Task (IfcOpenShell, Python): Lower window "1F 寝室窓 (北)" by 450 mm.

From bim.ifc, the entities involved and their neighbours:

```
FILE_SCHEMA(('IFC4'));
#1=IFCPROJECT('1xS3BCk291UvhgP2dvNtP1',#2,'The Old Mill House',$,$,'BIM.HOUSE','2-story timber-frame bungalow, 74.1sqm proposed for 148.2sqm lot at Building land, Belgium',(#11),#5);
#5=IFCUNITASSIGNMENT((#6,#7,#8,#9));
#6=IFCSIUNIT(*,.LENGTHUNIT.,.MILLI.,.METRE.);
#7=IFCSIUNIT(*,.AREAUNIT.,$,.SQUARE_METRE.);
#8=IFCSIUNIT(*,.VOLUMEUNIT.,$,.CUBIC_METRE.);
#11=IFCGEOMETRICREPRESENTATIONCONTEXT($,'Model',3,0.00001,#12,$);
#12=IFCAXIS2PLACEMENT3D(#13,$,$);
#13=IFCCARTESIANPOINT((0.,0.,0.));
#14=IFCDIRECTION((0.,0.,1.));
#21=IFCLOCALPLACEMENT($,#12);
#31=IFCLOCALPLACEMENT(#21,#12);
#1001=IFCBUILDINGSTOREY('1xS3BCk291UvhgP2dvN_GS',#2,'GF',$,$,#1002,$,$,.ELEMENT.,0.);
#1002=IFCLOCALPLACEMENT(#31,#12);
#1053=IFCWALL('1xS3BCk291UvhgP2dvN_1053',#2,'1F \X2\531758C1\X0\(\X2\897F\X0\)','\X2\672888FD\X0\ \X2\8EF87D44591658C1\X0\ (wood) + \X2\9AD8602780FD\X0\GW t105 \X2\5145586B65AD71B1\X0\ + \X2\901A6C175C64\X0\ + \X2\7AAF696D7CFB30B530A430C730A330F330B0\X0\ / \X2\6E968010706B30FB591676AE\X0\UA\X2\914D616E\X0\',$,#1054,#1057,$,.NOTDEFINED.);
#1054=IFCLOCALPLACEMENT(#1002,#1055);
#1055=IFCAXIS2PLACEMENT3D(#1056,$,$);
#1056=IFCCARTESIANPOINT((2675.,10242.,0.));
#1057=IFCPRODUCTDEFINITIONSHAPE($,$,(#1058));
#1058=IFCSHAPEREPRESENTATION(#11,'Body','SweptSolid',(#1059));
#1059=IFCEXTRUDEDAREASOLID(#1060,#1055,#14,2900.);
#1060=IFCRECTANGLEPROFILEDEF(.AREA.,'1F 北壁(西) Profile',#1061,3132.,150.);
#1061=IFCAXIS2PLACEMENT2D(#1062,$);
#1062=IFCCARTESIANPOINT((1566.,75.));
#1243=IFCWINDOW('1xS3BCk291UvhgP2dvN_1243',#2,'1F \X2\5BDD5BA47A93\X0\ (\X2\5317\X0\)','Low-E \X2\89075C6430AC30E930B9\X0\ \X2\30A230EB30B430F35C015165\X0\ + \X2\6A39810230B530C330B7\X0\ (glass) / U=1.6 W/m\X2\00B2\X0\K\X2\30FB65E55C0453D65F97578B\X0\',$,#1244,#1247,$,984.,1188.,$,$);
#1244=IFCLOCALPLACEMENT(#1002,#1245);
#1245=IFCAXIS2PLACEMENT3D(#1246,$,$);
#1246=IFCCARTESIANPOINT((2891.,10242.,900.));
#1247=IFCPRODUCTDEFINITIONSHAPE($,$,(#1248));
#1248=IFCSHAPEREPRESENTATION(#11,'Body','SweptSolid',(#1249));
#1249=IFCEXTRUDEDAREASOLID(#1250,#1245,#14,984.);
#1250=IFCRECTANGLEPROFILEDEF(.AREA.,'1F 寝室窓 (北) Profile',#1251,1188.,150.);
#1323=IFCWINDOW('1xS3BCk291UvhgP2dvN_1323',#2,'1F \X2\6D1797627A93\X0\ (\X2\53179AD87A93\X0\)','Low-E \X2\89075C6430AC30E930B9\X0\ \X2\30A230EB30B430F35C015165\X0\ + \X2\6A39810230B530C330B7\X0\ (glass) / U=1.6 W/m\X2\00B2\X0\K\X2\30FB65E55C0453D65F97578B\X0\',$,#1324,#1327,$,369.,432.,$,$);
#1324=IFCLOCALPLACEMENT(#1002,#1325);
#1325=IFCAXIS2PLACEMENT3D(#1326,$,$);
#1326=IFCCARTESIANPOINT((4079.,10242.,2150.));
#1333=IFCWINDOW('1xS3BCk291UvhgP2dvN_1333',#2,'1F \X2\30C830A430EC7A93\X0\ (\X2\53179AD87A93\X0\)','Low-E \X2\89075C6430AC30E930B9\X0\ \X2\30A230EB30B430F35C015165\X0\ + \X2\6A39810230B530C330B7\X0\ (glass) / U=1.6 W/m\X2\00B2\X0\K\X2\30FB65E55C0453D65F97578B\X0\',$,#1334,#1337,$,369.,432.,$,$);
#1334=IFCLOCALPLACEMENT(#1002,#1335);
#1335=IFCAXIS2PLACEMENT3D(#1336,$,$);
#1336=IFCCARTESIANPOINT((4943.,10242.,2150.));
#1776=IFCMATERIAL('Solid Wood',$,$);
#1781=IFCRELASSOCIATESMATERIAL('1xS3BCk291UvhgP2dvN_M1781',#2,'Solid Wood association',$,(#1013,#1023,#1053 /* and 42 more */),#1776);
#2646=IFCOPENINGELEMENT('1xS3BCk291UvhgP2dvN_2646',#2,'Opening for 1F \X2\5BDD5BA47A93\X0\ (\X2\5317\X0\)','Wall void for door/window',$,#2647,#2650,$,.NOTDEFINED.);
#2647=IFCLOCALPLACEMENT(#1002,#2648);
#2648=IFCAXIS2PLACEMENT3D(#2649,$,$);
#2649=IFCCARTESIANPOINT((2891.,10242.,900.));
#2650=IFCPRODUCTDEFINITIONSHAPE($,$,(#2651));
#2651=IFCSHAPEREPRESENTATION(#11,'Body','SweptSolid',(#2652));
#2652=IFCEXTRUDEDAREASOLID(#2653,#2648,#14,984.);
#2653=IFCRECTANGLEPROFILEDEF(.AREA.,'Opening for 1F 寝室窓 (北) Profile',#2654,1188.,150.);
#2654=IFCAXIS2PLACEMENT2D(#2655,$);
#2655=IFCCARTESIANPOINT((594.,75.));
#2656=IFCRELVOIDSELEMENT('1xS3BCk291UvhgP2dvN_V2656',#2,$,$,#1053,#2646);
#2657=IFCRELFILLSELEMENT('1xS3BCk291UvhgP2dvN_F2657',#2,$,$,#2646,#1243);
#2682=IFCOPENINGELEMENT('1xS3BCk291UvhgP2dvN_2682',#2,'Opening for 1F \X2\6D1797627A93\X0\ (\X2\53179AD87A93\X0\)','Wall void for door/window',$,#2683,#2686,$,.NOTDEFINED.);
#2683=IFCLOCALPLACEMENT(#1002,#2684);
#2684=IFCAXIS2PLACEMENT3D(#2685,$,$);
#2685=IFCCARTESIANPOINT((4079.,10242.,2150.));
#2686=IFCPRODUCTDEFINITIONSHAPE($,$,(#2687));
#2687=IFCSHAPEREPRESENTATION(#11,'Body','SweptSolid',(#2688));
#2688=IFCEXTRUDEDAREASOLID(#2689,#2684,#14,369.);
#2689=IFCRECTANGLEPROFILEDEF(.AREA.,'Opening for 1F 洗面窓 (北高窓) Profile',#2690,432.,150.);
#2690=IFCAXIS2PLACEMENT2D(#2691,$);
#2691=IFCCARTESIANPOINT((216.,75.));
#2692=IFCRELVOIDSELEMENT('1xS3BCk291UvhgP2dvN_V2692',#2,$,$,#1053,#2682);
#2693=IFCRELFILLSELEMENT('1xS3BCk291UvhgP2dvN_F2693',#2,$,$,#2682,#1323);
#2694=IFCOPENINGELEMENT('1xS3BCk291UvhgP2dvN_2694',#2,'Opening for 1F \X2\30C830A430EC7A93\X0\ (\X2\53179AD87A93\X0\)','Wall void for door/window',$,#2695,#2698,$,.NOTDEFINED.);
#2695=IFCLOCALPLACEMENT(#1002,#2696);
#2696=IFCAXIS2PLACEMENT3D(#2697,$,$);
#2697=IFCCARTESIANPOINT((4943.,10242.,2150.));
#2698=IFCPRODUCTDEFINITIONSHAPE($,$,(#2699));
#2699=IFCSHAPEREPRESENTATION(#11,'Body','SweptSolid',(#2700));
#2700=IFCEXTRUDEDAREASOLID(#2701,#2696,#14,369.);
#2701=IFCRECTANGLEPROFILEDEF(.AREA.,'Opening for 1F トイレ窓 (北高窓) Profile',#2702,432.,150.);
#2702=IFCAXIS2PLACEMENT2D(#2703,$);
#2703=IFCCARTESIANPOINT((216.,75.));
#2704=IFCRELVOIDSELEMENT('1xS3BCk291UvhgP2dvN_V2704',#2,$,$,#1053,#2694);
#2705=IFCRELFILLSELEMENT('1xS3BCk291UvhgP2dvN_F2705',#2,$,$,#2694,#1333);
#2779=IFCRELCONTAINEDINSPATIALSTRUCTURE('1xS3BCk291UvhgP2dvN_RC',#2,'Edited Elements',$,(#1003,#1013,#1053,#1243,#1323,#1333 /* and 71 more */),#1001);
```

```python
import numpy as np
import ifcopenshell
import ifcopenshell.api.geometry
import ifcopenshell.util.placement
import ifcopenshell.util.unit

model = ifcopenshell.open("bim.ifc")
unit_scale = ifcopenshell.util.unit.calculate_unit_scale(model)

window = model.by_id(1243)
opening = window.FillsVoids[0].RelatingOpeningElement
dz = -0.45 / unit_scale

shift = np.array([0.0, 0.0, dz])
# The window is not placed relative to its opening, so move both.
for product in (opening, window):
    matrix = ifcopenshell.util.placement.get_local_placement(product.ObjectPlacement)
    matrix[:3, 3] += shift
    ifcopenshell.api.geometry.edit_object_placement(model, product=product, matrix=matrix, is_si=False)

print(f"moved by {dz * unit_scale:+.3f} m")

model.write("bim_rev.ifc")
```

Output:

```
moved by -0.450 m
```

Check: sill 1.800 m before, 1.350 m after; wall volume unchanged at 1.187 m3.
